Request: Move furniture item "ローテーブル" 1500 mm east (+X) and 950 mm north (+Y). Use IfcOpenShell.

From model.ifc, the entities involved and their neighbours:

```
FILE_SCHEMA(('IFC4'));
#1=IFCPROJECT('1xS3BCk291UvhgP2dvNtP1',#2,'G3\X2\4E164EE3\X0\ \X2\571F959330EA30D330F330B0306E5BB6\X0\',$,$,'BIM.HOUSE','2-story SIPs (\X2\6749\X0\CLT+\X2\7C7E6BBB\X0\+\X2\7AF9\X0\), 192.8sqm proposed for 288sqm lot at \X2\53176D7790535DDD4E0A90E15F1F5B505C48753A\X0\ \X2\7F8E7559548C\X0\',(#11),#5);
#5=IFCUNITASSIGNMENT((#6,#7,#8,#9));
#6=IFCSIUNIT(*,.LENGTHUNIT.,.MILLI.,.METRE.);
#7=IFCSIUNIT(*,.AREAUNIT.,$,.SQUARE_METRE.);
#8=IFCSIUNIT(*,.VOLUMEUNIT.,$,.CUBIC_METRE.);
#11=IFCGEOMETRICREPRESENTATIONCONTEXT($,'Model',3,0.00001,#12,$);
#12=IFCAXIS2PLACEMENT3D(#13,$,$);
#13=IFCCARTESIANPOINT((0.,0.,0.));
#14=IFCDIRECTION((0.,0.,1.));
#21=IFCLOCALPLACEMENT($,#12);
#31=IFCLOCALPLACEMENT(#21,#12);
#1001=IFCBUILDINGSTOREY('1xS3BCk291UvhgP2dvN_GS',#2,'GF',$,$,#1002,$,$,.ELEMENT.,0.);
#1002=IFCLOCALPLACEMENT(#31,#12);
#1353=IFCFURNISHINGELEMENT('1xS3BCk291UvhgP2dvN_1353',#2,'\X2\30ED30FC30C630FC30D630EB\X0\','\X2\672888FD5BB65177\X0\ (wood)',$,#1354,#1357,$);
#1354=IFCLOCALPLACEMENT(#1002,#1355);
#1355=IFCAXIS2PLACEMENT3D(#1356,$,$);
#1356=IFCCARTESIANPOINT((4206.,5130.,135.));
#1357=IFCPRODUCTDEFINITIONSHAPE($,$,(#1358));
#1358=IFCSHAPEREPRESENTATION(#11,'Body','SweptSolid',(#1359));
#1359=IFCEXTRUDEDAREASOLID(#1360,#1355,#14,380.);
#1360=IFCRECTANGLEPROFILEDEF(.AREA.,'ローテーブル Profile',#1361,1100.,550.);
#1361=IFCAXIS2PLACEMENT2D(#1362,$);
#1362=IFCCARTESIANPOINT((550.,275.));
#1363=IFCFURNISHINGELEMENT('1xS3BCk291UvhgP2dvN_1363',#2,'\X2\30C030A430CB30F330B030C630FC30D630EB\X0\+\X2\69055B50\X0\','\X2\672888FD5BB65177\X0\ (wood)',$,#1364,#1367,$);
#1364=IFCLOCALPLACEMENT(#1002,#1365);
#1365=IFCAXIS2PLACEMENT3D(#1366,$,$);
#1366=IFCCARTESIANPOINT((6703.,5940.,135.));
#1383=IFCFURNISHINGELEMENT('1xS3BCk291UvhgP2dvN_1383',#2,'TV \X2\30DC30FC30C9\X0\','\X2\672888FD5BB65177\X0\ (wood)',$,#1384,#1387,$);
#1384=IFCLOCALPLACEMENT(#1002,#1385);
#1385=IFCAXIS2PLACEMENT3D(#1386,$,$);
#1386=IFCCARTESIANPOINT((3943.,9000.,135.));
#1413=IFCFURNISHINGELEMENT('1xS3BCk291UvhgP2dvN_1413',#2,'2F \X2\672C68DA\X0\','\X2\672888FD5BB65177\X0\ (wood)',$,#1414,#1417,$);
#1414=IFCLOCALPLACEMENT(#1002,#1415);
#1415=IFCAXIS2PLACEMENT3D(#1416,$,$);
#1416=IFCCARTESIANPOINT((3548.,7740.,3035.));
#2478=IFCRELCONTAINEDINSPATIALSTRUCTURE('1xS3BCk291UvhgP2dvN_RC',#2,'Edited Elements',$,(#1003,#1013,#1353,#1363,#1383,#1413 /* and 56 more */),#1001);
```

```python
import ifcopenshell
import ifcopenshell.api.geometry
import ifcopenshell.util.placement
import ifcopenshell.util.unit

model = ifcopenshell.open("model.ifc")
unit_scale = ifcopenshell.util.unit.calculate_unit_scale(model)

item = model.by_id(1353)
matrix = ifcopenshell.util.placement.get_local_placement(item.ObjectPlacement)
matrix[0, 3] += 1.5 / unit_scale
matrix[1, 3] += 0.95 / unit_scale
ifcopenshell.api.geometry.edit_object_placement(model, product=item, matrix=matrix, is_si=False)

print(ifcopenshell.util.placement.get_local_placement(item.ObjectPlacement).round(3) + 0.0)

model.write("model-out.ifc")
```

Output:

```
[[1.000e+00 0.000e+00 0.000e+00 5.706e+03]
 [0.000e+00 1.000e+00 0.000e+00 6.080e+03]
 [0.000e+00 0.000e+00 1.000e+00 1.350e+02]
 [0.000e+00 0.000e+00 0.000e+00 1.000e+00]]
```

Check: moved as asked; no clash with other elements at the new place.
